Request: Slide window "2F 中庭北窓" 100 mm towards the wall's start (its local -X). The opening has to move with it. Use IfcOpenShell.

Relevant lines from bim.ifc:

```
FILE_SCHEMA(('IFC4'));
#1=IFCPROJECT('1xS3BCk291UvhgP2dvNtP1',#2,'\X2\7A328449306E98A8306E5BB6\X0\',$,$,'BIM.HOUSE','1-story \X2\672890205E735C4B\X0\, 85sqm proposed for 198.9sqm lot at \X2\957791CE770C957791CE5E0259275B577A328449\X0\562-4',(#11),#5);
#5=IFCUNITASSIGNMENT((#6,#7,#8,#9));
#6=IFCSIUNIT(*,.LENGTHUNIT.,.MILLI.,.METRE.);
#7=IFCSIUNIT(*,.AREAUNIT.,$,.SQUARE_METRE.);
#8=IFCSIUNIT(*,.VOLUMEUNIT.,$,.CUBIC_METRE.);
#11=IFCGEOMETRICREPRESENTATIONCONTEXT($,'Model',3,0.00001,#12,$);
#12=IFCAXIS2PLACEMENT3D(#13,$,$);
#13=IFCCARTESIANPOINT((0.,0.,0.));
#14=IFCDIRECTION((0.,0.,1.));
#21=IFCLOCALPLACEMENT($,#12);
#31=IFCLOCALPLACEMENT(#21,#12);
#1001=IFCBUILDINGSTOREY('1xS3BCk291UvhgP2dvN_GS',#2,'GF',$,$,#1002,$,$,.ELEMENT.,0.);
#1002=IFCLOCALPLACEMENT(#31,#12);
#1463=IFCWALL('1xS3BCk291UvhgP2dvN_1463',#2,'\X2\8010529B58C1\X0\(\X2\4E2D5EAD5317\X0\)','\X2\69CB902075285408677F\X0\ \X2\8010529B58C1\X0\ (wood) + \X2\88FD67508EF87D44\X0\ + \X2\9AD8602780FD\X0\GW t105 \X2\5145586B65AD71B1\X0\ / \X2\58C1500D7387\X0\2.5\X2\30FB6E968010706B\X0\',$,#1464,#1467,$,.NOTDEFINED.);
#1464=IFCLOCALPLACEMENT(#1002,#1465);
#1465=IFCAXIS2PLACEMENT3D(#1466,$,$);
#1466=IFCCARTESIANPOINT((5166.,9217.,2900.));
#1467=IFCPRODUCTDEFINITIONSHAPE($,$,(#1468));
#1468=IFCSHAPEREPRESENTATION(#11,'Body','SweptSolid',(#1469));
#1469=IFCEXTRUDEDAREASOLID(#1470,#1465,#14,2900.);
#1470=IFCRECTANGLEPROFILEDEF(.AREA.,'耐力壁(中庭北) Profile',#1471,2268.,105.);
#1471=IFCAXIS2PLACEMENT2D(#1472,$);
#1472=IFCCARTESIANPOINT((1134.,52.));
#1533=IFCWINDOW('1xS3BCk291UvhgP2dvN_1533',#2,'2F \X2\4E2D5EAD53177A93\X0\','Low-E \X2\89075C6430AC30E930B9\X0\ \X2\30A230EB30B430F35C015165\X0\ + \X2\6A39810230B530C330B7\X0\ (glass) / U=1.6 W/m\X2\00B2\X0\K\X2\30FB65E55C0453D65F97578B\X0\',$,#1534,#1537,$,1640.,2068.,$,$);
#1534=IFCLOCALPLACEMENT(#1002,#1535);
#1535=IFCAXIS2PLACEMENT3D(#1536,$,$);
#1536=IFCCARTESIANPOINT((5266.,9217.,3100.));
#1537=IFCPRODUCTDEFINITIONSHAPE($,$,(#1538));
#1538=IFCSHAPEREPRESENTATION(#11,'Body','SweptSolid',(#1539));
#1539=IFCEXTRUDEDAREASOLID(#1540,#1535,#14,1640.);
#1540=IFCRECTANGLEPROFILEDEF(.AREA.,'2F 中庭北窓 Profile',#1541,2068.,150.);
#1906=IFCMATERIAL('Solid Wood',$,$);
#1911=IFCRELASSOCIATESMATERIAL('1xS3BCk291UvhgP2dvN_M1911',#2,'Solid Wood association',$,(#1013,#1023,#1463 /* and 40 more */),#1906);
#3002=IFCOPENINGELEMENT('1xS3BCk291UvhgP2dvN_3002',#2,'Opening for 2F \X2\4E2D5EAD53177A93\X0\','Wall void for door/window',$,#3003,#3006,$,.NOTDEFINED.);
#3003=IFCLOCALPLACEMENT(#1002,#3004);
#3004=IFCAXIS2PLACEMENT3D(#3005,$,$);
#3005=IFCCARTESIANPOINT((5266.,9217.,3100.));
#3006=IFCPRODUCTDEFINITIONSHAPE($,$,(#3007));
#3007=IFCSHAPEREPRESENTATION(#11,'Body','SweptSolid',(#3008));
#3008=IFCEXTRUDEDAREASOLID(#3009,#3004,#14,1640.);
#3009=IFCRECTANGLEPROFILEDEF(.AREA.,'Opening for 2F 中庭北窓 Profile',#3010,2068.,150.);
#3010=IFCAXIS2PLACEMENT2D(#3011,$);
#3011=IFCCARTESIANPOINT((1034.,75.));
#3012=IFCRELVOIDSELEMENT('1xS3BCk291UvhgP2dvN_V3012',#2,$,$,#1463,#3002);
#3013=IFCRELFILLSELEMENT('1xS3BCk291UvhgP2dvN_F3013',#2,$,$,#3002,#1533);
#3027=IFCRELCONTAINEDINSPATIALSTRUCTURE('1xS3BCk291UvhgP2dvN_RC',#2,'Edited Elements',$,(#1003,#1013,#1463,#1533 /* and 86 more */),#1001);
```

```python
import ifcopenshell
import ifcopenshell.api.geometry
import ifcopenshell.util.placement

model = ifcopenshell.open("bim.ifc")

window = model.by_guid("1xS3BCk291UvhgP2dvN_1533")
opening = window.FillsVoids[0].RelatingOpeningElement
wall = opening.VoidsElements[0].RelatingBuildingElement

wall_matrix = ifcopenshell.util.placement.get_local_placement(wall.ObjectPlacement)
shift = wall_matrix[:3, 0] * -100.0
before = ifcopenshell.util.placement.get_local_placement(window.ObjectPlacement)[:3, 3].copy()

# The window is not placed relative to its opening, so move both.
for product in (opening, window):
    matrix = ifcopenshell.util.placement.get_local_placement(product.ObjectPlacement)
    matrix[:3, 3] += shift
    ifcopenshell.api.geometry.edit_object_placement(model, product=product, matrix=matrix, is_si=False)

after = ifcopenshell.util.placement.get_local_placement(window.ObjectPlacement)[:3, 3]
print("window moved by", (after - before).round(3) + 0.0)

model.write("bim_edited.ifc")
```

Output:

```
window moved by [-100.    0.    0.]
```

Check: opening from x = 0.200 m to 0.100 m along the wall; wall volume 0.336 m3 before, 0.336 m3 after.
